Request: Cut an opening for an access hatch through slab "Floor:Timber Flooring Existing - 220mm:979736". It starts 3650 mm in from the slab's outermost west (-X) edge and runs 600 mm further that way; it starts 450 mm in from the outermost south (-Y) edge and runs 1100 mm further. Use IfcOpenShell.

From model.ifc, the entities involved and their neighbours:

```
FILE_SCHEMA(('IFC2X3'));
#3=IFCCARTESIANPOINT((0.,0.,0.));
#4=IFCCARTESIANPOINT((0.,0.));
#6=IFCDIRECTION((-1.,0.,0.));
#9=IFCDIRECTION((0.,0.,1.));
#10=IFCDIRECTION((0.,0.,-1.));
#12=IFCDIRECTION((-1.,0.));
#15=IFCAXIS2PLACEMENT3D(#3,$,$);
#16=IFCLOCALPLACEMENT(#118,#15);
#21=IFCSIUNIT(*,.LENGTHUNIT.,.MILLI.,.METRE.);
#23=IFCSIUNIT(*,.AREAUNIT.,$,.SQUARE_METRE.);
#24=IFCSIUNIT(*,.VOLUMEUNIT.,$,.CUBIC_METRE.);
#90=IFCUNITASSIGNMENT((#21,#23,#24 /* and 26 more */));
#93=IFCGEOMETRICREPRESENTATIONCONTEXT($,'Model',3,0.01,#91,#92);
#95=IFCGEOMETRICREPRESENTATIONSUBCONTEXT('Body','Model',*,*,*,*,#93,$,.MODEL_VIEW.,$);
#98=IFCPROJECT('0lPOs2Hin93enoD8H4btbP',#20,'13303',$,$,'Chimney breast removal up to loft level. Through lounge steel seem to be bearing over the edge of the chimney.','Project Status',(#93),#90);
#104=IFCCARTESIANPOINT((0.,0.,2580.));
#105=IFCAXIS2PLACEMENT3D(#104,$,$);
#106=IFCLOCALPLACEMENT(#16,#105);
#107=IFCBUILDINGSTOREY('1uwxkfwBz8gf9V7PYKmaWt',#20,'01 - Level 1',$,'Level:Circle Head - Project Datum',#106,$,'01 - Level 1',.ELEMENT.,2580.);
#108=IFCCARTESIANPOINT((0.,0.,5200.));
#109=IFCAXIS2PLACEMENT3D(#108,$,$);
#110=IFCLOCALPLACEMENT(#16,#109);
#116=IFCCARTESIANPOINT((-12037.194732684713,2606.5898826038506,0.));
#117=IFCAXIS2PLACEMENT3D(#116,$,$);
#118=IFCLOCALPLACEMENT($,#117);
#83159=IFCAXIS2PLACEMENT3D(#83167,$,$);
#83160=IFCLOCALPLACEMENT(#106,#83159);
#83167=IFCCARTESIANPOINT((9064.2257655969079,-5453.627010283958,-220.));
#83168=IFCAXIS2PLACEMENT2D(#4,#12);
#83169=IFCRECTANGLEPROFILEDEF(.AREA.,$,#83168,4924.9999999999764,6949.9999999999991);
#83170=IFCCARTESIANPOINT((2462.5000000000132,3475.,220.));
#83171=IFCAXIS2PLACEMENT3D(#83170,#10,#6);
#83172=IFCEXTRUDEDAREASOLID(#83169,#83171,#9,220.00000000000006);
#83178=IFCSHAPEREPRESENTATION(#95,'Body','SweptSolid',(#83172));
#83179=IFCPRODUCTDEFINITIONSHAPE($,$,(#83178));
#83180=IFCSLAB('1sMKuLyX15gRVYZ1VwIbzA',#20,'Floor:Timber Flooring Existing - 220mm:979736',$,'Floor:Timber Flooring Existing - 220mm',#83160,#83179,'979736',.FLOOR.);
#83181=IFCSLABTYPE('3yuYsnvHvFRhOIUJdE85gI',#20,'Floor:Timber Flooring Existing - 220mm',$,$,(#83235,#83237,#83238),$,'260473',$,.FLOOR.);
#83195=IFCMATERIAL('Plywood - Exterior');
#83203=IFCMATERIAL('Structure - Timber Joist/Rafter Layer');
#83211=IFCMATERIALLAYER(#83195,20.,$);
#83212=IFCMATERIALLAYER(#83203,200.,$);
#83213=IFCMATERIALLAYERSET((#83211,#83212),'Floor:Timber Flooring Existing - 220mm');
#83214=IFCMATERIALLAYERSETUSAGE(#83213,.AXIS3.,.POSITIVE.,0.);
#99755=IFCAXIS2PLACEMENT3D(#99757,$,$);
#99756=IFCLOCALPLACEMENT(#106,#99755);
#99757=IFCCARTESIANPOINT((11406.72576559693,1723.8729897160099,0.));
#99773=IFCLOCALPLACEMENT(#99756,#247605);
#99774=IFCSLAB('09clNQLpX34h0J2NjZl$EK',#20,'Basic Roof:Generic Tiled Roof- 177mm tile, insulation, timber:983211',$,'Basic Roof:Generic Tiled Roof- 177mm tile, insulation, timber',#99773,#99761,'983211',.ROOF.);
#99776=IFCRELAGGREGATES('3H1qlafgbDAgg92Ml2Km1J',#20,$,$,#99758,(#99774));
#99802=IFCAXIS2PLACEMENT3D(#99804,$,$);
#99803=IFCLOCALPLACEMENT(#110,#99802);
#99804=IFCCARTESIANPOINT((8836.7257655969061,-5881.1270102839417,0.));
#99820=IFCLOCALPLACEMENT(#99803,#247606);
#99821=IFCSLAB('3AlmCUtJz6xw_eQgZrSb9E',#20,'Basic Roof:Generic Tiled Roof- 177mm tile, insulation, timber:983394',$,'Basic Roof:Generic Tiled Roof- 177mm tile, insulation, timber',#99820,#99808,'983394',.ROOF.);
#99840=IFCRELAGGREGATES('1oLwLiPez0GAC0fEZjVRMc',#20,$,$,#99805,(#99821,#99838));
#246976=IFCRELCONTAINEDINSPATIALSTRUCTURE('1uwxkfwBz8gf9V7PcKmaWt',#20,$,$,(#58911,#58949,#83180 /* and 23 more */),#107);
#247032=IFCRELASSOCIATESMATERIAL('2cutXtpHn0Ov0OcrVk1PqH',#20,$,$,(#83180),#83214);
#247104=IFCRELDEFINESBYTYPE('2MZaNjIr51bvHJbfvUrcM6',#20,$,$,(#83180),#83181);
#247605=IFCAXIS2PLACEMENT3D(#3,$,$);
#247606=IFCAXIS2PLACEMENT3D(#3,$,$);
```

```python
import numpy as np
import ifcopenshell
import ifcopenshell.api.feature
import ifcopenshell.api.geometry
import ifcopenshell.api.root
import ifcopenshell.geom
import ifcopenshell.util.placement
import ifcopenshell.util.representation
import ifcopenshell.util.shape
import ifcopenshell.util.unit

model = ifcopenshell.open("model.ifc")
unit_scale = ifcopenshell.util.unit.calculate_unit_scale(model)
settings = ifcopenshell.geom.settings()


def volume(element):
    """Net volume in cubic metres, openings subtracted."""
    shape = ifcopenshell.geom.create_shape(settings, element)
    return ifcopenshell.util.shape.get_volume(shape.geometry)


slab = model.by_id(83180)
before = volume(slab)

# Extent in the slab's own axes, in metres. The edges named are its -X and -Y sides.
slab_shape = ifcopenshell.geom.create_shape(settings, slab)
vertices = ifcopenshell.util.shape.get_vertices(slab_shape.geometry)
x_min, y_min, bottom = vertices.min(axis=0)
top = vertices[:, 2].max()

opening = ifcopenshell.api.root.create_entity(model, ifc_class="IfcOpeningElement", name="Access hatch opening")
context = ifcopenshell.util.representation.get_context(model, "Model", "Body", "MODEL_VIEW")
width, depth = 0.6, 1.1
outline = [(0.0, 0.0), (width, 0.0), (width, depth), (0.0, depth), (0.0, 0.0)]
# Overshoot both faces by 50 mm so the cut is clean.
shape = ifcopenshell.api.geometry.add_slab_representation(
    model, context=context, depth=top - bottom + 0.1, polyline=outline
)
ifcopenshell.api.geometry.assign_representation(model, product=opening, representation=shape)

matrix = ifcopenshell.util.placement.get_local_placement(slab.ObjectPlacement)
matrix[:, 3] = matrix @ np.append(np.array([x_min + 3.65, y_min + 0.45, bottom - 0.05]) / unit_scale, 1.0)
ifcopenshell.api.geometry.edit_object_placement(model, product=opening, matrix=matrix, is_si=False)
ifcopenshell.api.feature.add_feature(model, feature=opening, element=slab)

after = volume(slab)

print(f"slab volume {before:.3f} -> {after:.3f} m3")

model.write("model_rev.ifc")
```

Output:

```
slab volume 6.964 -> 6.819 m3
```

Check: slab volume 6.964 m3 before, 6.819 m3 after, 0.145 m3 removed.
